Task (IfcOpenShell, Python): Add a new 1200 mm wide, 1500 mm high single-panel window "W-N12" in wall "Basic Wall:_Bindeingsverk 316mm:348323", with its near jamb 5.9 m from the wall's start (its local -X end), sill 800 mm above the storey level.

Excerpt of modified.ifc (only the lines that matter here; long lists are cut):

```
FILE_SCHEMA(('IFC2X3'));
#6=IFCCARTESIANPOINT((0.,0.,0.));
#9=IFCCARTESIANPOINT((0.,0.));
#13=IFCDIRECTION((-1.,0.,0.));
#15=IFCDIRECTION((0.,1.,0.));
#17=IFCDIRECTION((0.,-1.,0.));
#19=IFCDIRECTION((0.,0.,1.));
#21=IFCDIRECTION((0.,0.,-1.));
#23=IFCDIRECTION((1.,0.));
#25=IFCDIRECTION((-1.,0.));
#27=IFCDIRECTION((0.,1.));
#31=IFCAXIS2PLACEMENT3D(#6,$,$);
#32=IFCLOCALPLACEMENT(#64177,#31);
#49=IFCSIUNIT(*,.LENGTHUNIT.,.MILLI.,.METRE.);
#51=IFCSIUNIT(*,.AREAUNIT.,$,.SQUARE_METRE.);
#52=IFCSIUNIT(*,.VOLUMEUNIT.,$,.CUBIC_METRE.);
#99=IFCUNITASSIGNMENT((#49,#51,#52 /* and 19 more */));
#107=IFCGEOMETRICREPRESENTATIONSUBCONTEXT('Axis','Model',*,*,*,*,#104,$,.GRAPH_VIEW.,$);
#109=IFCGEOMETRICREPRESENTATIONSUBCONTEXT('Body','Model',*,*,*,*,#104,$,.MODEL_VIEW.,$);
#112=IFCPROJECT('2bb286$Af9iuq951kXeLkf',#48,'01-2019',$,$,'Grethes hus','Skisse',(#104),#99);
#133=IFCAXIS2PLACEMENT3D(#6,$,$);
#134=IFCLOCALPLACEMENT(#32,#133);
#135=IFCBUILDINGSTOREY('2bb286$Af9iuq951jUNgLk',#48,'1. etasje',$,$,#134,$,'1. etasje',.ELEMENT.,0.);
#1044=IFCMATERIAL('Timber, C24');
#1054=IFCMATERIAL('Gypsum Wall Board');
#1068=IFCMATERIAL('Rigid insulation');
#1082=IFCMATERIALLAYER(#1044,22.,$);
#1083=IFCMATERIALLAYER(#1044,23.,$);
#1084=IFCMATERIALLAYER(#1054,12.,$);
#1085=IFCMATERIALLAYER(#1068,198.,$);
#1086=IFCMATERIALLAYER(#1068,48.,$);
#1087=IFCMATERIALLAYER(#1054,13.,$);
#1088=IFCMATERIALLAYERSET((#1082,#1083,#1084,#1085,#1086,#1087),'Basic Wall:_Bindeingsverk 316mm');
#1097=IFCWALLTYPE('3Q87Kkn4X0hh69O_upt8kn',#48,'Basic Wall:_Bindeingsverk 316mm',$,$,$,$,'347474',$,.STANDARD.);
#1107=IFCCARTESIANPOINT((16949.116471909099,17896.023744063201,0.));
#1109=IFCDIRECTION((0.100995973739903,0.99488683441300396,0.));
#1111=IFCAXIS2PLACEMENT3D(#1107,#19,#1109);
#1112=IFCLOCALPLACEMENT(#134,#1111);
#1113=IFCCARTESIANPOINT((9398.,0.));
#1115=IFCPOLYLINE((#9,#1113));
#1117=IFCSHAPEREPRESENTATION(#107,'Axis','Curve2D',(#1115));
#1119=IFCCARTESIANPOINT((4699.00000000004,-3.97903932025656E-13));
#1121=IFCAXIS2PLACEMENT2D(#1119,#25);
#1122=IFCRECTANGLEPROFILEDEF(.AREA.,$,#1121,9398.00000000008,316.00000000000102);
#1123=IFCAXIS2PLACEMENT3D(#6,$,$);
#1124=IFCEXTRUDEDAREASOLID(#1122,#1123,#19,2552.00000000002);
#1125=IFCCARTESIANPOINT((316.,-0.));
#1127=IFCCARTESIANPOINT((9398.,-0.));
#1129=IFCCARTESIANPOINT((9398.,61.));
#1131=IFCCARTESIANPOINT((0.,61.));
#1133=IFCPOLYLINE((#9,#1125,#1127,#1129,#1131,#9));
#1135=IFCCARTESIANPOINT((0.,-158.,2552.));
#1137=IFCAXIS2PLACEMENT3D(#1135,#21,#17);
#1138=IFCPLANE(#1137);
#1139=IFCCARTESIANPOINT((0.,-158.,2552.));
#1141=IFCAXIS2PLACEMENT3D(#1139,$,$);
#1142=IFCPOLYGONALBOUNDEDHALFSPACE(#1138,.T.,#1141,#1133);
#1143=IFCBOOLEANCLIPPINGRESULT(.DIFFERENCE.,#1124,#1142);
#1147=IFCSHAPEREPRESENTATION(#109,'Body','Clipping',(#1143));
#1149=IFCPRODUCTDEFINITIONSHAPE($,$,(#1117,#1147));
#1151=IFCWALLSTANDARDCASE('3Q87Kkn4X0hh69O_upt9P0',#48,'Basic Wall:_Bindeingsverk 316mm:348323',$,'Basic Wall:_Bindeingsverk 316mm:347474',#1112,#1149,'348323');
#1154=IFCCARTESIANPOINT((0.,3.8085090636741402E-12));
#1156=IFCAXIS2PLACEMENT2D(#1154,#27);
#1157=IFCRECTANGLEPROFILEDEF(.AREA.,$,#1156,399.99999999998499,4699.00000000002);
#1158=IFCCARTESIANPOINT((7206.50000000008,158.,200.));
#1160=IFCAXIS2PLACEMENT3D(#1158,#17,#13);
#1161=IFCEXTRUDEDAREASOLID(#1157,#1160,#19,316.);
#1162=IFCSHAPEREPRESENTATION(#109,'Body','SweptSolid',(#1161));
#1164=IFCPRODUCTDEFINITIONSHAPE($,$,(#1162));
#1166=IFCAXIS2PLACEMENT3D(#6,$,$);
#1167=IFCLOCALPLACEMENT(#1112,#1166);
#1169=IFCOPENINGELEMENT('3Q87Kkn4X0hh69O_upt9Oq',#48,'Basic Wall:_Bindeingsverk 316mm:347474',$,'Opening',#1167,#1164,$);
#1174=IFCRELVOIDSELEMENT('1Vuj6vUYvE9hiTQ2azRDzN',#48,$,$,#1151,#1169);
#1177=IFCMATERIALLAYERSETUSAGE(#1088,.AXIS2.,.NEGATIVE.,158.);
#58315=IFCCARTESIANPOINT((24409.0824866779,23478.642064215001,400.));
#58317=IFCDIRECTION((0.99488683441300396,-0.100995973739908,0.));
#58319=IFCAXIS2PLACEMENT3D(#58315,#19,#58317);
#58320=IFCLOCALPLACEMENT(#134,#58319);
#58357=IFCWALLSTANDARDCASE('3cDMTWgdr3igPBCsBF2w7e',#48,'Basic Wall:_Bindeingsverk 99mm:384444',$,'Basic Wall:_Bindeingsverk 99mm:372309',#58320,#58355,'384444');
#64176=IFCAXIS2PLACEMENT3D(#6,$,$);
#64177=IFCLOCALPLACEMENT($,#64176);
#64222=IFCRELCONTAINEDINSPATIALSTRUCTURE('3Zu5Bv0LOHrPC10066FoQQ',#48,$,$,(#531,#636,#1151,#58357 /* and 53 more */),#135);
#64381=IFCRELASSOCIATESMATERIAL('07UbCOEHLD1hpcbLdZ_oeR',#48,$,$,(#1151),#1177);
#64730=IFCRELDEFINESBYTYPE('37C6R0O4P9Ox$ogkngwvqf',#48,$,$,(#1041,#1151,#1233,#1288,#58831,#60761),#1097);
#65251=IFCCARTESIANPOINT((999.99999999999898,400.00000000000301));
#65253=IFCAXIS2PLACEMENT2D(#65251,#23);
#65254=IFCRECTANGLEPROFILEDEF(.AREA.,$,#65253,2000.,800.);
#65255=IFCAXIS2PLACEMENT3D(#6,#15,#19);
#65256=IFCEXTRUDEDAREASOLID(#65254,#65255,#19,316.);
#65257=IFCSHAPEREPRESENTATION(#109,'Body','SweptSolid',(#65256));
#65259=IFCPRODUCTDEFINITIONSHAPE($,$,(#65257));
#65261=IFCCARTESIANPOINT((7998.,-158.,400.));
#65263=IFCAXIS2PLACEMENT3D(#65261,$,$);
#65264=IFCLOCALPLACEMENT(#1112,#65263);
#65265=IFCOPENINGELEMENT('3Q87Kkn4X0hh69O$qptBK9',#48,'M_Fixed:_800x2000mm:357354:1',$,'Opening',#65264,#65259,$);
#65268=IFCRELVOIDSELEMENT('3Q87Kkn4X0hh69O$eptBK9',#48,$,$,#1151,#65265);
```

```python
import numpy as np
import ifcopenshell
import ifcopenshell.api.feature
import ifcopenshell.api.geometry
import ifcopenshell.api.root
import ifcopenshell.api.spatial
import ifcopenshell.api.type
import ifcopenshell.geom
import ifcopenshell.util.element
import ifcopenshell.util.placement
import ifcopenshell.util.representation
import ifcopenshell.util.shape
import ifcopenshell.util.unit

model = ifcopenshell.open("modified.ifc")
unit_scale = ifcopenshell.util.unit.calculate_unit_scale(model)
settings = ifcopenshell.geom.settings()


def volume(element):
    """Net volume in cubic metres, openings subtracted."""
    shape = ifcopenshell.geom.create_shape(settings, element)
    return ifcopenshell.util.shape.get_volume(shape.geometry)


wall = model.by_guid("3Q87Kkn4X0hh69O_upt9P0")
storey = ifcopenshell.util.element.get_container(wall, ifc_class="IfcBuildingStorey")
context = ifcopenshell.util.representation.get_context(model, "Model", "Body", "MODEL_VIEW")
before = volume(wall)

width, height, from_end, sill = 1.2, 1.5, 5.9, 0.8  # metres

# The wall runs along its own X axis, and the end named is its -X end.
wall_shape = ifcopenshell.geom.create_shape(settings, wall)
x, y, z = ifcopenshell.util.shape.get_vertices(wall_shape.geometry).T
start = x.min() + from_end
face, thickness = float(y.min()), float(y.max() - y.min())
wall_matrix = ifcopenshell.util.placement.get_local_placement(wall.ObjectPlacement)
level = ifcopenshell.util.placement.get_local_placement(storey.ObjectPlacement)[2, 3]


def in_wall(x, y):
    """Placement at x, y metres in the wall's axes, at sill height."""
    matrix = wall_matrix.copy()
    matrix[:, 3] = wall_matrix @ np.array([x / unit_scale, y / unit_scale, 0.0, 1.0])
    matrix[2, 3] = level + sill / unit_scale
    return matrix


# Opening: a box that overshoots both wall faces by 50 mm.
opening = ifcopenshell.api.root.create_entity(model, ifc_class="IfcOpeningElement")
box = ifcopenshell.api.geometry.add_wall_representation(
    model, context=context, length=width, height=height, thickness=thickness + 0.1
)
ifcopenshell.api.geometry.assign_representation(model, product=opening, representation=box)
ifcopenshell.api.geometry.edit_object_placement(model, product=opening, matrix=in_wall(start, face - 0.05), is_si=False)
ifcopenshell.api.feature.add_feature(model, feature=opening, element=wall)

window = ifcopenshell.api.root.create_entity(model, ifc_class="IfcWindow", name="W-N12")
window.OverallWidth, window.OverallHeight = width / unit_scale, height / unit_scale
body = ifcopenshell.api.geometry.add_window_representation(
    model,
    context=context,
    overall_width=window.OverallWidth,
    overall_height=window.OverallHeight,
    partition_type="SINGLE_PANEL",
)
ifcopenshell.api.geometry.assign_representation(model, product=window, representation=body)
ifcopenshell.api.spatial.assign_container(model, products=[window], relating_structure=storey)
fills = ifcopenshell.api.feature.add_filling(model, opening=opening, element=window)
fills.OwnerHistory = window.OwnerHistory  # required in IFC2X3

# IFC2X3 keeps the operation on the window style.
style = ifcopenshell.api.root.create_entity(model, ifc_class="IfcWindowStyle", name="W-N12")
style.OperationType, style.ConstructionType = "SINGLE_PANEL", "NOTDEFINED"
style.ParameterTakesPrecedence = style.Sizeable = False
ifcopenshell.api.type.assign_type(model, related_objects=[window], relating_type=style)

# Centre the window in the wall's thickness.
ifcopenshell.api.geometry.edit_object_placement(model, product=window, matrix=in_wall(start, face), is_si=False)
window_shape = ifcopenshell.geom.create_shape(settings, window)
depth = ifcopenshell.util.shape.get_vertices(window_shape.geometry)[:, 1]
offset = face + thickness / 2 - (depth.min() + depth.max()) / 2
ifcopenshell.api.geometry.edit_object_placement(model, product=window, matrix=in_wall(start, offset), is_si=False)

after = volume(wall)

print(f"wall volume {before:.3f} -> {after:.3f} m3")

model.write("modified-out.ifc")
```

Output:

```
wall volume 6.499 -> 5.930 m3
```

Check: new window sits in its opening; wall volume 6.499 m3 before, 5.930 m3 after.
